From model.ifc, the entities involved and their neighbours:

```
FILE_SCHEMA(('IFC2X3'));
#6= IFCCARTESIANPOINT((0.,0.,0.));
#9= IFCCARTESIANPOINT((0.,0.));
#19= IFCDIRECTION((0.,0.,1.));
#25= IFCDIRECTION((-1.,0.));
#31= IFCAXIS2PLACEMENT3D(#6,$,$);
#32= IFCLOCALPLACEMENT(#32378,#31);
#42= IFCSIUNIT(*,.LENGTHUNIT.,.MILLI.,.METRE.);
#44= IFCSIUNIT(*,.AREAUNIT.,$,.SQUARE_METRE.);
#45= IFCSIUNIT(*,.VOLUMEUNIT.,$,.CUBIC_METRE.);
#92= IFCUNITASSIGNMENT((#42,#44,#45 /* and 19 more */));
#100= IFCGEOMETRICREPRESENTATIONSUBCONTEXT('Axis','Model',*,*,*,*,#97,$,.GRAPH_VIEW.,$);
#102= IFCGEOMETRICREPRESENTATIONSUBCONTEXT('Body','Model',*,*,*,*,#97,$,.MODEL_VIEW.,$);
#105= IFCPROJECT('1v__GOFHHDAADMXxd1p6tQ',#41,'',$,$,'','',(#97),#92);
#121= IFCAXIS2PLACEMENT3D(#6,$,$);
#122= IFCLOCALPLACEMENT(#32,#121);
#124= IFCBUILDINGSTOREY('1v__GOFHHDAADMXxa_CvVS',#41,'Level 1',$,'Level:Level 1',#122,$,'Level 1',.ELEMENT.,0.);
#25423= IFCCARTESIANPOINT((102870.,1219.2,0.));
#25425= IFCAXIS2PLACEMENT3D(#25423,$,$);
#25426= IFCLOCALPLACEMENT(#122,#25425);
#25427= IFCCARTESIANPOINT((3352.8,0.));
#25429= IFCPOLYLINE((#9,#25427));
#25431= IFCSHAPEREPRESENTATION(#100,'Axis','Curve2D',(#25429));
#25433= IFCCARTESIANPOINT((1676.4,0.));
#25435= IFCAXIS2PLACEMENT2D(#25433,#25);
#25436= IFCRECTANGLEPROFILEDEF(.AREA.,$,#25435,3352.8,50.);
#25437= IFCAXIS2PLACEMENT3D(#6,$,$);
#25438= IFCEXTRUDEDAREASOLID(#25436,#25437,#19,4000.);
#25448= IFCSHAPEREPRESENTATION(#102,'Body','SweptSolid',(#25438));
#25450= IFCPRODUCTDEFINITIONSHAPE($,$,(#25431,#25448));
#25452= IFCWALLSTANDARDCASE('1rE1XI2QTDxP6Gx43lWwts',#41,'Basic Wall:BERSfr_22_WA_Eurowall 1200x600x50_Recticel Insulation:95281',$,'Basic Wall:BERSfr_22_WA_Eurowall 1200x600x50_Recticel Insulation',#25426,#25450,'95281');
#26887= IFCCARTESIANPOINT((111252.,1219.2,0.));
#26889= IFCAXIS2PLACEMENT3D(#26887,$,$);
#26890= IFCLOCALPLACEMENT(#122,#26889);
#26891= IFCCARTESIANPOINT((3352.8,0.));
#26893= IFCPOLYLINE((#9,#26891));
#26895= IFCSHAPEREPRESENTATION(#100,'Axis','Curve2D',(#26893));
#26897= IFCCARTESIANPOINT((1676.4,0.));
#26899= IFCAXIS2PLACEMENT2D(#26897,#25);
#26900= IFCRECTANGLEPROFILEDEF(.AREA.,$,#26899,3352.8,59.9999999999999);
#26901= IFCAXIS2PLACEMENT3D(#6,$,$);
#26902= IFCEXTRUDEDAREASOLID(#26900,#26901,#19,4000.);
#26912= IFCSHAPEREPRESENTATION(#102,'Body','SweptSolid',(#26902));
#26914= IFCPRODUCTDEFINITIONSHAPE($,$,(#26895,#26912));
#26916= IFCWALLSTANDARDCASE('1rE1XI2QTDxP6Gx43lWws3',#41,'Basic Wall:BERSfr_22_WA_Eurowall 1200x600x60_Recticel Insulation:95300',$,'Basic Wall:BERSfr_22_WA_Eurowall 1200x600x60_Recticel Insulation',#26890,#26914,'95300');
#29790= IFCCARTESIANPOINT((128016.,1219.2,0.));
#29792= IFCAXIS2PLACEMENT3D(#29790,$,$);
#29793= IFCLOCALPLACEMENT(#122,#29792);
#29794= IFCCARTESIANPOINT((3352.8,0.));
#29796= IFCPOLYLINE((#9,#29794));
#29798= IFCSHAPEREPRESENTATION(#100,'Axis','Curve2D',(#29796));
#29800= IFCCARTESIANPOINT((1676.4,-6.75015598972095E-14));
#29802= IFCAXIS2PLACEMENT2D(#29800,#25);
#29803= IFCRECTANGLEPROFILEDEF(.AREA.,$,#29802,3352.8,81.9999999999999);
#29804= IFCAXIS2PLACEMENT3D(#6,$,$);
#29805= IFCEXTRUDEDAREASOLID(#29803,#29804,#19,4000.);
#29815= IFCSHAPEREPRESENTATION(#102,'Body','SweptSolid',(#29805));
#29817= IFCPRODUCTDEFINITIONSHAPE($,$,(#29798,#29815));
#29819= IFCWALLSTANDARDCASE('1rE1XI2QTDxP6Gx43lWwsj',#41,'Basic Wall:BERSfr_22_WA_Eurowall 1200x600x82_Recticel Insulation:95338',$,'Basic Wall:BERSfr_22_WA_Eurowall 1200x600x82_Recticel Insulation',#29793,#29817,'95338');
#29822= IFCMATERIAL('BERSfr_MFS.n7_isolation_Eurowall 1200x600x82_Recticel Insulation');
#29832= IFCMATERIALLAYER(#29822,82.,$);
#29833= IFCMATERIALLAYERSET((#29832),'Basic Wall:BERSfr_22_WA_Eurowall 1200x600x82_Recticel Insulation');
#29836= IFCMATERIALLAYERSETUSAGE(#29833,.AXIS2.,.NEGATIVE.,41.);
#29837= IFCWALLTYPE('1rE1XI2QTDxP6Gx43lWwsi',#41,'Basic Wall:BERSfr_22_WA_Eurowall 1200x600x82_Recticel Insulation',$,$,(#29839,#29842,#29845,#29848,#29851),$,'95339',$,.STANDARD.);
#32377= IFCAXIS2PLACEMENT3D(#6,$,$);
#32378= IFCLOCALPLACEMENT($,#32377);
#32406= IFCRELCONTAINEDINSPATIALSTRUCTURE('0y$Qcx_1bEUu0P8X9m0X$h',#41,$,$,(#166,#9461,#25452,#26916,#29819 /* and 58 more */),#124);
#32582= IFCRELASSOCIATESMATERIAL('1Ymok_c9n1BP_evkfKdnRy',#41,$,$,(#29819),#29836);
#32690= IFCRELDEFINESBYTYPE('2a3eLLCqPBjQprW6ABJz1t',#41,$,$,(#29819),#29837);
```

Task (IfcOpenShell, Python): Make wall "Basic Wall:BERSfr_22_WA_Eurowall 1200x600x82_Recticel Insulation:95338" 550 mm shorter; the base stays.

```python
import ifcopenshell
import ifcopenshell.geom
import ifcopenshell.util.representation
import ifcopenshell.util.shape
import ifcopenshell.util.unit

model = ifcopenshell.open("model.ifc")
unit_scale = ifcopenshell.util.unit.calculate_unit_scale(model)
settings = ifcopenshell.geom.settings()


def volume(element):
    """Net volume in cubic metres, openings subtracted."""
    shape = ifcopenshell.geom.create_shape(settings, element)
    return ifcopenshell.util.shape.get_volume(shape.geometry)


wall = model.by_guid("1rE1XI2QTDxP6Gx43lWwsj")
before = volume(wall)

body = ifcopenshell.util.representation.get_representation(wall, "Model", "Body")
solid = body.Items[0]
old_height = solid.Depth
solid.Depth -= 0.55 / unit_scale
after = volume(wall)

print(f"height {old_height:g} -> {solid.Depth:g}, volume {before:.3f} -> {after:.3f} m3")

model.write("model_rev.ifc")
```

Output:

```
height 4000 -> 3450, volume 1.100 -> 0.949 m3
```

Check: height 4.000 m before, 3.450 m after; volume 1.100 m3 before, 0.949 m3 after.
